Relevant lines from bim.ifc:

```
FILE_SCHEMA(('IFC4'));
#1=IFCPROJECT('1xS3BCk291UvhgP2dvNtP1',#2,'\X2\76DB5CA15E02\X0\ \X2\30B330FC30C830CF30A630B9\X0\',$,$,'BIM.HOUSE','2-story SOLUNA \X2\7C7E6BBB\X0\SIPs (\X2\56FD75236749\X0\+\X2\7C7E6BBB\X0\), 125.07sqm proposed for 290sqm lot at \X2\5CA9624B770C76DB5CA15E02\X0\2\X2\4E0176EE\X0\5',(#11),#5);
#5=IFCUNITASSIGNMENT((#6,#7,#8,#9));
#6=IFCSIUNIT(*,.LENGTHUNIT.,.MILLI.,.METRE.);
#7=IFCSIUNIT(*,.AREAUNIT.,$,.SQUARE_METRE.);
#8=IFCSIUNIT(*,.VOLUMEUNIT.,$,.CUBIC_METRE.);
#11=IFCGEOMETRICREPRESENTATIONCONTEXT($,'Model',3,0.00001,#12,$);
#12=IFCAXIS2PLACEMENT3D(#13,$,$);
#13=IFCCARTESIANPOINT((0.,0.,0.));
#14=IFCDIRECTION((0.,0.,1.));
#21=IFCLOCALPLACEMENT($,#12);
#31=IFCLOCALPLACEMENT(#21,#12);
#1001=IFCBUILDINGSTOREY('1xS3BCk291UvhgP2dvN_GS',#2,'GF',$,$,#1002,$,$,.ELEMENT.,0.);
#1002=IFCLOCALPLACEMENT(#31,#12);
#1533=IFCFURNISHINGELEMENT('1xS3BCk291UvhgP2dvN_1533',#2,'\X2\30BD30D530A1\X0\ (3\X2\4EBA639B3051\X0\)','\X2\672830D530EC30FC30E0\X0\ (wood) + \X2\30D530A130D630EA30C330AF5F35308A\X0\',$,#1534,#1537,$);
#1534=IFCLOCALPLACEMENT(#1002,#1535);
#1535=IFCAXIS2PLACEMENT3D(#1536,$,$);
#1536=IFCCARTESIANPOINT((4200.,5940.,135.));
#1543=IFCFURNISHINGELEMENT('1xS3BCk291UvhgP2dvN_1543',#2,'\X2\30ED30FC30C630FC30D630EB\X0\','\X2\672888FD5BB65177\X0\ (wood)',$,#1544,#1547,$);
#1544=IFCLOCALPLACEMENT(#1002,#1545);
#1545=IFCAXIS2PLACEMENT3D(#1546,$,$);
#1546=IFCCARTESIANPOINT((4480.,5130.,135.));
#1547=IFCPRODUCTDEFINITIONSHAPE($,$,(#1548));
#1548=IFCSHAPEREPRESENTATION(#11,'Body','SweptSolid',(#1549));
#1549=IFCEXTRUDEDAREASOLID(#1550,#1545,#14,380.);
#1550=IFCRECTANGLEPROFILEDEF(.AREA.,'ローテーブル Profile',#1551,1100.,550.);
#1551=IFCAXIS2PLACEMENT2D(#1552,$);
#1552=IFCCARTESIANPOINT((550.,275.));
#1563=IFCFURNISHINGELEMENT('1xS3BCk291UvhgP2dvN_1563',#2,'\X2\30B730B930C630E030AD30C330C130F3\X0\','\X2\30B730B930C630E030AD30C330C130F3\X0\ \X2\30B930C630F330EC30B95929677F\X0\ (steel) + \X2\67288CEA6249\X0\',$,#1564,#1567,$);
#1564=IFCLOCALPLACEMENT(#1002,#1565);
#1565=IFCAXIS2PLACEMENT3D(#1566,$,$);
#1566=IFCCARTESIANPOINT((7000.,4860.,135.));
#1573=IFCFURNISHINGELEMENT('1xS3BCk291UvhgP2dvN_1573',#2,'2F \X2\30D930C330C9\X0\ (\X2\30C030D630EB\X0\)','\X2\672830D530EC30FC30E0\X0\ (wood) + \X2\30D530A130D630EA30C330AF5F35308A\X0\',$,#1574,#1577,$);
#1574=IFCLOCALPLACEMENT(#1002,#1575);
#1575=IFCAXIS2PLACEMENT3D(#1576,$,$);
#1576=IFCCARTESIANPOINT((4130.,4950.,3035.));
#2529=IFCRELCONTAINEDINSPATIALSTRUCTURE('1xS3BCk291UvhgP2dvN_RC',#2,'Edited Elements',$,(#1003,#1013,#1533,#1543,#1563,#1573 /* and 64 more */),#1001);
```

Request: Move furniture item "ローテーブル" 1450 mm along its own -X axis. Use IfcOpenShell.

```python
import ifcopenshell
import ifcopenshell.api.geometry
import ifcopenshell.util.placement
import ifcopenshell.util.unit

model = ifcopenshell.open("bim.ifc")
unit_scale = ifcopenshell.util.unit.calculate_unit_scale(model)

item = model.by_guid("1xS3BCk291UvhgP2dvN_1543")
matrix = ifcopenshell.util.placement.get_local_placement(item.ObjectPlacement)
matrix[:3, 3] -= matrix[:3, 0] * 1.45 / unit_scale
ifcopenshell.api.geometry.edit_object_placement(model, product=item, matrix=matrix, is_si=False)

print(ifcopenshell.util.placement.get_local_placement(item.ObjectPlacement).round(3) + 0.0)

model.write("bim_rev.ifc")
```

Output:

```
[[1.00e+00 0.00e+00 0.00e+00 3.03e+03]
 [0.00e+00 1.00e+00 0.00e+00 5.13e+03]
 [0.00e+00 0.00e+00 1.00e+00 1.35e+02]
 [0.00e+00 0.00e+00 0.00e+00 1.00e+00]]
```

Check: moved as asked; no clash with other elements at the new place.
